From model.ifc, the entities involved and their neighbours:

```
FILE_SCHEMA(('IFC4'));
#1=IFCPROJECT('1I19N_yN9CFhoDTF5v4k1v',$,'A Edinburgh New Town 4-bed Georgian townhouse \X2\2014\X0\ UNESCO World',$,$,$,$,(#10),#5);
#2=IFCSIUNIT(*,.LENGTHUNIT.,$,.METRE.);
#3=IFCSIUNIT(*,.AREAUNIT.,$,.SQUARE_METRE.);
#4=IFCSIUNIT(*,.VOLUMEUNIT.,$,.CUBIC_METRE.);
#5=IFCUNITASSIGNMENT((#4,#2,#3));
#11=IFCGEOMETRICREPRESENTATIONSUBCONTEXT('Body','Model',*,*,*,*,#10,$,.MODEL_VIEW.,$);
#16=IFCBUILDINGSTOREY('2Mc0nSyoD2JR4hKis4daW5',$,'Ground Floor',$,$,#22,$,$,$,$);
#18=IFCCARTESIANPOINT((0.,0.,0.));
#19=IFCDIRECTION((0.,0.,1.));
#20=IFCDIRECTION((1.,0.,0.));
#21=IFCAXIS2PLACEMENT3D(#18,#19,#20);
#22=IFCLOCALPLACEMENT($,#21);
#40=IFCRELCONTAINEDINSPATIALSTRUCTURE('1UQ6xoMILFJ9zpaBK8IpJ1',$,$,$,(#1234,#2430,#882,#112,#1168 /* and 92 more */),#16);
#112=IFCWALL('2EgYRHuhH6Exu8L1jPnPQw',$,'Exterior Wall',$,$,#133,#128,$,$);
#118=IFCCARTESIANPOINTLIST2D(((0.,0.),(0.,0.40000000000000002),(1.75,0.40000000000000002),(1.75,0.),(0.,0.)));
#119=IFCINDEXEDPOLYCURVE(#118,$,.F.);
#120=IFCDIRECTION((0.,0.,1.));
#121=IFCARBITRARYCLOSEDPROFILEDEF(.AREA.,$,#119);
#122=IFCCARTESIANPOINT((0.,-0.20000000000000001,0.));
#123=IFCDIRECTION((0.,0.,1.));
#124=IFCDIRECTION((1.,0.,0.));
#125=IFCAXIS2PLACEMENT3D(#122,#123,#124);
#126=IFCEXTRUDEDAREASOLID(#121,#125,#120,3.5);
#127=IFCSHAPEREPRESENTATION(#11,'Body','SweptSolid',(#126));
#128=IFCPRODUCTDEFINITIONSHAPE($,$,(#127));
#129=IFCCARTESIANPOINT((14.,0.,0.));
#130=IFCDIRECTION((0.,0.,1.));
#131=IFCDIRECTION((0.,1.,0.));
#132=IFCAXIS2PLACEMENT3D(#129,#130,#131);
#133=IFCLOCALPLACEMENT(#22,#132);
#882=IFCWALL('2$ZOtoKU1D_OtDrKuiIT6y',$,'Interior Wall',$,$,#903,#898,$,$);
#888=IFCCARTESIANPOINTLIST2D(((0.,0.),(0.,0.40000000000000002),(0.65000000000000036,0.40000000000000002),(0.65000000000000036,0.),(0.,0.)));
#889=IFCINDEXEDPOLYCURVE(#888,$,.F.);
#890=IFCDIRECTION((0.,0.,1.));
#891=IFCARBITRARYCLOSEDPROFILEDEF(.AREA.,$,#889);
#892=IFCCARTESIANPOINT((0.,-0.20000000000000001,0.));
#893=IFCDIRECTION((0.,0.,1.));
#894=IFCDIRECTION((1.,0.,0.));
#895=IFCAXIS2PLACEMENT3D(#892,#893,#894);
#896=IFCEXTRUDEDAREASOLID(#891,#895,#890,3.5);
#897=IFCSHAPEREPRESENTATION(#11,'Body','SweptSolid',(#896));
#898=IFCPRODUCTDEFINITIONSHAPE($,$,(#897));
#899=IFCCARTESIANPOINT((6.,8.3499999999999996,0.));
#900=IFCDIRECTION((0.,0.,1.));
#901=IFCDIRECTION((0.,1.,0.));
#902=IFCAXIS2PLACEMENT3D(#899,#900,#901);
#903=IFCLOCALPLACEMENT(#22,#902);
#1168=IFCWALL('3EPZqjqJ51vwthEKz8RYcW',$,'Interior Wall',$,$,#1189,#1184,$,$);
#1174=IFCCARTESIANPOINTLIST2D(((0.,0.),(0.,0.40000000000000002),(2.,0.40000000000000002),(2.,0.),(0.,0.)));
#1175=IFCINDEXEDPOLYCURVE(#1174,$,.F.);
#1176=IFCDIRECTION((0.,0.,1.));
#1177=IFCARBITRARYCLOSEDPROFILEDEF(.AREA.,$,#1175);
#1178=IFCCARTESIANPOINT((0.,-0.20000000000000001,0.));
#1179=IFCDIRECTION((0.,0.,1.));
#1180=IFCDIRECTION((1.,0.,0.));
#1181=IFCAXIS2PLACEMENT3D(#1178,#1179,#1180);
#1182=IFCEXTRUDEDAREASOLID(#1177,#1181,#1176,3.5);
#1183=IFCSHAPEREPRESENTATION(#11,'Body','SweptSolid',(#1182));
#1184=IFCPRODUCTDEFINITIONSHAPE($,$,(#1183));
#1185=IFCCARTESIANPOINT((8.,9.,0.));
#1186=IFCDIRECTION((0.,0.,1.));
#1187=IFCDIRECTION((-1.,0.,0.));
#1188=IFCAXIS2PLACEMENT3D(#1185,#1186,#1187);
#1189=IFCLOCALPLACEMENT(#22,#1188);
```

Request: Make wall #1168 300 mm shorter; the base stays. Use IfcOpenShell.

```python
import ifcopenshell
import ifcopenshell.geom
import ifcopenshell.util.representation
import ifcopenshell.util.shape
import ifcopenshell.util.unit

model = ifcopenshell.open("model.ifc")
unit_scale = ifcopenshell.util.unit.calculate_unit_scale(model)
settings = ifcopenshell.geom.settings()


def volume(element):
    """Net volume in cubic metres, openings subtracted."""
    shape = ifcopenshell.geom.create_shape(settings, element)
    return ifcopenshell.util.shape.get_volume(shape.geometry)


wall = model.by_guid("3EPZqjqJ51vwthEKz8RYcW")
before = volume(wall)

body = ifcopenshell.util.representation.get_representation(wall, "Model", "Body")
solid = body.Items[0]
old_height = solid.Depth
solid.Depth -= 0.3 / unit_scale
after = volume(wall)

print(f"height {old_height:g} -> {solid.Depth:g}, volume {before:.3f} -> {after:.3f} m3")

model.write("model_v2.ifc")
```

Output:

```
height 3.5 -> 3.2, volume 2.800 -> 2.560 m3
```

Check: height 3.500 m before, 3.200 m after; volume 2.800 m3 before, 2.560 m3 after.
